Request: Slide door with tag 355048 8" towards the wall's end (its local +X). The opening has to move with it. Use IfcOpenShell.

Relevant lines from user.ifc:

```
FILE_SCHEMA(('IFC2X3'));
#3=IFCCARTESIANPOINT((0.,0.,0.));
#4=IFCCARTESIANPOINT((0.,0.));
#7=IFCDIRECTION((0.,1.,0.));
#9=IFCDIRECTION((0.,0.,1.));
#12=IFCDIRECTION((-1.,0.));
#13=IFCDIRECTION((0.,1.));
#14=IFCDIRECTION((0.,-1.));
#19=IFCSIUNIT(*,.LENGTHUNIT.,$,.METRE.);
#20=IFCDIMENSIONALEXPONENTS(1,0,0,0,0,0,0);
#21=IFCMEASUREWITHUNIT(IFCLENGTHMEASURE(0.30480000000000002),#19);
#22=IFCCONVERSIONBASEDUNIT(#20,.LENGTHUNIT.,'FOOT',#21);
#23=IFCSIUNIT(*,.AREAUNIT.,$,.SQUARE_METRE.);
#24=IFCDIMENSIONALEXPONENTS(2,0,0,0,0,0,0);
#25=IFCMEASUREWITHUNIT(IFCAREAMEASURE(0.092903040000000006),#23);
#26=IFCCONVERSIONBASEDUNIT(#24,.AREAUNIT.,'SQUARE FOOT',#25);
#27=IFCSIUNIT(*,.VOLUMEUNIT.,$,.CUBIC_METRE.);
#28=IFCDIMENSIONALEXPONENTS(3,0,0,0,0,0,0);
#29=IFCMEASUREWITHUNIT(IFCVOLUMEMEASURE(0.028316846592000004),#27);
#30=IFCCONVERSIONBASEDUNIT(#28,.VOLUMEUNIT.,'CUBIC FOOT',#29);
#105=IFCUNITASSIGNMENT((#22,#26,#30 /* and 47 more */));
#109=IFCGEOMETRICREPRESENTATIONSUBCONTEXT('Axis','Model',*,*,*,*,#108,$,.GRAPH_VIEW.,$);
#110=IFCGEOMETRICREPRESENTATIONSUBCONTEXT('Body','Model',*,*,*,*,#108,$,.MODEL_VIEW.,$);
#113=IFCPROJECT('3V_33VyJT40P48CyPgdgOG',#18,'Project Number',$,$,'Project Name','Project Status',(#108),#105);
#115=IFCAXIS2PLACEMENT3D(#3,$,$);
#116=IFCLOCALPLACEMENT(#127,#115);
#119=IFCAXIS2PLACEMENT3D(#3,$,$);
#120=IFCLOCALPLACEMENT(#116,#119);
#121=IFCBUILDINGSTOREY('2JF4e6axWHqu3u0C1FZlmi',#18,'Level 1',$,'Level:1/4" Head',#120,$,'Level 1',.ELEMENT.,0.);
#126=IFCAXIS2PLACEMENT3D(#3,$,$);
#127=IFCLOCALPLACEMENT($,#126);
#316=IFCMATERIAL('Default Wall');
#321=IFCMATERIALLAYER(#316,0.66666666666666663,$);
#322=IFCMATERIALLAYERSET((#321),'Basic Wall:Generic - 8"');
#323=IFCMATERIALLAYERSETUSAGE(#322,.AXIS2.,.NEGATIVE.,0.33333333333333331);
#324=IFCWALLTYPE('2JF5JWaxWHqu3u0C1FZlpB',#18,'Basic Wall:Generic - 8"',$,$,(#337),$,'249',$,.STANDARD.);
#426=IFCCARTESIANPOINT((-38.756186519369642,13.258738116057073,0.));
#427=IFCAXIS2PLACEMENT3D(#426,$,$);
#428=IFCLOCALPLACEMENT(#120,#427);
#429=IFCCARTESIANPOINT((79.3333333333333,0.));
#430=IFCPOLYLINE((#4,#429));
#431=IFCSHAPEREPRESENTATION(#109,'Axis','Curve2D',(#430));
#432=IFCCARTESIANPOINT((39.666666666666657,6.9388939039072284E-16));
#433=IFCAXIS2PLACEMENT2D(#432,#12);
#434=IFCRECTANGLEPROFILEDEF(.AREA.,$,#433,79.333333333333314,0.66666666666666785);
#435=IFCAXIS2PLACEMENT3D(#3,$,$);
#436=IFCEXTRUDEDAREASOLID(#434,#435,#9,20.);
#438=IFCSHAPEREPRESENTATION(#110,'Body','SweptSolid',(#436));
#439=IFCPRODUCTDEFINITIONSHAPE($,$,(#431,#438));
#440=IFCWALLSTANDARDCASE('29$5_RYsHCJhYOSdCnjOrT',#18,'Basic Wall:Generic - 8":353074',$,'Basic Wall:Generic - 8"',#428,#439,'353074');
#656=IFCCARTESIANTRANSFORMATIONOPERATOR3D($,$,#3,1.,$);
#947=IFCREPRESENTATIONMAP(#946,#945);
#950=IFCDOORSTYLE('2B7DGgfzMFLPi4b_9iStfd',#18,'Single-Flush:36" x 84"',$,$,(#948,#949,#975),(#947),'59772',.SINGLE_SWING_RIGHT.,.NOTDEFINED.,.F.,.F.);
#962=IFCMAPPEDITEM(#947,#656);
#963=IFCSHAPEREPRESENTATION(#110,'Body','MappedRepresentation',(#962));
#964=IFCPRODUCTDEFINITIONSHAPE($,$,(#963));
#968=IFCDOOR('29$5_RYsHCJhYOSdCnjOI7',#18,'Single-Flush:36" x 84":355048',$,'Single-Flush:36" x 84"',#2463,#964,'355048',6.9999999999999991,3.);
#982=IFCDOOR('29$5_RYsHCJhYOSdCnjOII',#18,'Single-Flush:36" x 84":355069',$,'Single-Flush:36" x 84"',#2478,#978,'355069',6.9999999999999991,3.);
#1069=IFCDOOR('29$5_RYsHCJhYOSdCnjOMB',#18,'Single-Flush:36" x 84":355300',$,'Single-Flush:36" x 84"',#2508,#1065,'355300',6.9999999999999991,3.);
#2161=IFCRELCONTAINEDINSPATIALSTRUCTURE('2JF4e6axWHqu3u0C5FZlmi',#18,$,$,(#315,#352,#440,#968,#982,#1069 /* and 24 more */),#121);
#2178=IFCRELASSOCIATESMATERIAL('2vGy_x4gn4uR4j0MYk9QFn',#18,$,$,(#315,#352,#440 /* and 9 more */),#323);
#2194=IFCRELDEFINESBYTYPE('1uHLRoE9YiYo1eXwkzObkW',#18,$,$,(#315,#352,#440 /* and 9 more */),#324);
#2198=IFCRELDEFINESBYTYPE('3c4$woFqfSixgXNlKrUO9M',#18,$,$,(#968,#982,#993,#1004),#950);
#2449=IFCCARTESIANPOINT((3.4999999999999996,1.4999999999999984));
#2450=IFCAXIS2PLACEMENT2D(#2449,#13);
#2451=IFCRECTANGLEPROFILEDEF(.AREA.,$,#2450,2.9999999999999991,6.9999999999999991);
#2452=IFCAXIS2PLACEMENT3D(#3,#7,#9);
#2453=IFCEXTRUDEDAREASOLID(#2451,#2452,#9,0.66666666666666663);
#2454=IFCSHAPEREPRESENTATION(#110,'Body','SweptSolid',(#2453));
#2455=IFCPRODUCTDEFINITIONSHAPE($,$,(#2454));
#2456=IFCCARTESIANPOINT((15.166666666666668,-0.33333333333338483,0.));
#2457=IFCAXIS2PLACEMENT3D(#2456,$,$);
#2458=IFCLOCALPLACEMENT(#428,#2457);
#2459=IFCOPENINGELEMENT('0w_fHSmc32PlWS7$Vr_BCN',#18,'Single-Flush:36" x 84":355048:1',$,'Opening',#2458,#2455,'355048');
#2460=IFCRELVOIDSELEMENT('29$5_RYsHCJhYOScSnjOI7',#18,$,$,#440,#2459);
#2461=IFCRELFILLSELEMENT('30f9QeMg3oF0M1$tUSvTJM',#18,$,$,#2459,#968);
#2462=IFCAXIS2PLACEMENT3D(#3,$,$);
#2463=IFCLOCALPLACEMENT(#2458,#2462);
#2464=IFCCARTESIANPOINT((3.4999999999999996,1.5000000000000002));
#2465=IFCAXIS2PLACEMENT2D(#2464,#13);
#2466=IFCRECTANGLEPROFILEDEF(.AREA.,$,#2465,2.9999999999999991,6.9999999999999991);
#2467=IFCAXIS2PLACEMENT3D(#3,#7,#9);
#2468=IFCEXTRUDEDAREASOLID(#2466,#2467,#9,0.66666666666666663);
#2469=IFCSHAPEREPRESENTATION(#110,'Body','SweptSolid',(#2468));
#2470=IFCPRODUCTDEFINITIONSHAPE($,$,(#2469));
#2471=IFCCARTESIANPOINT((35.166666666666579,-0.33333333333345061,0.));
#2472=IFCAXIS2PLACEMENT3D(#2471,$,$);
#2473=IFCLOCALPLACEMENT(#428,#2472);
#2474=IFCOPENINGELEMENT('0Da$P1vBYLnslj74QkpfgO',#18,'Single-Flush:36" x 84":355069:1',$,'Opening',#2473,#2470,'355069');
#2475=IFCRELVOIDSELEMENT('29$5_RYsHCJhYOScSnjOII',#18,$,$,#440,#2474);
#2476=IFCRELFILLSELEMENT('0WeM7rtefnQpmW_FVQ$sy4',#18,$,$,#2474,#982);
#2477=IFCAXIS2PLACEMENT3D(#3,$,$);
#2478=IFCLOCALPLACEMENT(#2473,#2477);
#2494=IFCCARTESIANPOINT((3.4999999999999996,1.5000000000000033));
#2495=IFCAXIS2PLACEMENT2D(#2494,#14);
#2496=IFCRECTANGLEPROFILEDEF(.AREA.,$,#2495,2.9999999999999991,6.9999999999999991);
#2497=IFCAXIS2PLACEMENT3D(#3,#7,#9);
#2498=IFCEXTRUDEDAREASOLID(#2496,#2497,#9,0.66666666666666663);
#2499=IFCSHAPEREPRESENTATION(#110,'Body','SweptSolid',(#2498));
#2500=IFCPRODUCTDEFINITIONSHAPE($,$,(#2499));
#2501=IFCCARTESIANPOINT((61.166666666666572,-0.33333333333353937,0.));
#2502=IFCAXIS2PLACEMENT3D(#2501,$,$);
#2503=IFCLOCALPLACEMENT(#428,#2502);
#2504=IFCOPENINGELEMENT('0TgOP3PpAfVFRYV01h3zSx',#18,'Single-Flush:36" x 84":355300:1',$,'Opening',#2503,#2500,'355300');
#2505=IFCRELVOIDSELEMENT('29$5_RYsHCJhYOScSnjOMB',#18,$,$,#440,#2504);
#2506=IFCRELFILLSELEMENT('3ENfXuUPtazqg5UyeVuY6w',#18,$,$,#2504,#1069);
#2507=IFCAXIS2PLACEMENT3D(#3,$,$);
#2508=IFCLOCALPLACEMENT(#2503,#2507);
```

```python
import ifcopenshell
import ifcopenshell.api.geometry
import ifcopenshell.util.placement
import ifcopenshell.util.unit

model = ifcopenshell.open("user.ifc")
unit_scale = ifcopenshell.util.unit.calculate_unit_scale(model)

door = model.by_id(968)
opening = door.FillsVoids[0].RelatingOpeningElement
wall = opening.VoidsElements[0].RelatingBuildingElement

wall_matrix = ifcopenshell.util.placement.get_local_placement(wall.ObjectPlacement)
shift = wall_matrix[:3, 0] * 8 * 0.0254 / unit_scale
before = ifcopenshell.util.placement.get_local_placement(door.ObjectPlacement)[:3, 3].copy()

# The door is placed relative to its opening, so it follows when the opening moves.
matrix = ifcopenshell.util.placement.get_local_placement(opening.ObjectPlacement)
matrix[:3, 3] += shift
ifcopenshell.api.geometry.edit_object_placement(
    model, product=opening, matrix=matrix, is_si=False, should_transform_children=True
)

after = ifcopenshell.util.placement.get_local_placement(door.ObjectPlacement)[:3, 3]
print("door moved by", (after - before).round(3) + 0.0)

model.write("user_edited.ifc")
```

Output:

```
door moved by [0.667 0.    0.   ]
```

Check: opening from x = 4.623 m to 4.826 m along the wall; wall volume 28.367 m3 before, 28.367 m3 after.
